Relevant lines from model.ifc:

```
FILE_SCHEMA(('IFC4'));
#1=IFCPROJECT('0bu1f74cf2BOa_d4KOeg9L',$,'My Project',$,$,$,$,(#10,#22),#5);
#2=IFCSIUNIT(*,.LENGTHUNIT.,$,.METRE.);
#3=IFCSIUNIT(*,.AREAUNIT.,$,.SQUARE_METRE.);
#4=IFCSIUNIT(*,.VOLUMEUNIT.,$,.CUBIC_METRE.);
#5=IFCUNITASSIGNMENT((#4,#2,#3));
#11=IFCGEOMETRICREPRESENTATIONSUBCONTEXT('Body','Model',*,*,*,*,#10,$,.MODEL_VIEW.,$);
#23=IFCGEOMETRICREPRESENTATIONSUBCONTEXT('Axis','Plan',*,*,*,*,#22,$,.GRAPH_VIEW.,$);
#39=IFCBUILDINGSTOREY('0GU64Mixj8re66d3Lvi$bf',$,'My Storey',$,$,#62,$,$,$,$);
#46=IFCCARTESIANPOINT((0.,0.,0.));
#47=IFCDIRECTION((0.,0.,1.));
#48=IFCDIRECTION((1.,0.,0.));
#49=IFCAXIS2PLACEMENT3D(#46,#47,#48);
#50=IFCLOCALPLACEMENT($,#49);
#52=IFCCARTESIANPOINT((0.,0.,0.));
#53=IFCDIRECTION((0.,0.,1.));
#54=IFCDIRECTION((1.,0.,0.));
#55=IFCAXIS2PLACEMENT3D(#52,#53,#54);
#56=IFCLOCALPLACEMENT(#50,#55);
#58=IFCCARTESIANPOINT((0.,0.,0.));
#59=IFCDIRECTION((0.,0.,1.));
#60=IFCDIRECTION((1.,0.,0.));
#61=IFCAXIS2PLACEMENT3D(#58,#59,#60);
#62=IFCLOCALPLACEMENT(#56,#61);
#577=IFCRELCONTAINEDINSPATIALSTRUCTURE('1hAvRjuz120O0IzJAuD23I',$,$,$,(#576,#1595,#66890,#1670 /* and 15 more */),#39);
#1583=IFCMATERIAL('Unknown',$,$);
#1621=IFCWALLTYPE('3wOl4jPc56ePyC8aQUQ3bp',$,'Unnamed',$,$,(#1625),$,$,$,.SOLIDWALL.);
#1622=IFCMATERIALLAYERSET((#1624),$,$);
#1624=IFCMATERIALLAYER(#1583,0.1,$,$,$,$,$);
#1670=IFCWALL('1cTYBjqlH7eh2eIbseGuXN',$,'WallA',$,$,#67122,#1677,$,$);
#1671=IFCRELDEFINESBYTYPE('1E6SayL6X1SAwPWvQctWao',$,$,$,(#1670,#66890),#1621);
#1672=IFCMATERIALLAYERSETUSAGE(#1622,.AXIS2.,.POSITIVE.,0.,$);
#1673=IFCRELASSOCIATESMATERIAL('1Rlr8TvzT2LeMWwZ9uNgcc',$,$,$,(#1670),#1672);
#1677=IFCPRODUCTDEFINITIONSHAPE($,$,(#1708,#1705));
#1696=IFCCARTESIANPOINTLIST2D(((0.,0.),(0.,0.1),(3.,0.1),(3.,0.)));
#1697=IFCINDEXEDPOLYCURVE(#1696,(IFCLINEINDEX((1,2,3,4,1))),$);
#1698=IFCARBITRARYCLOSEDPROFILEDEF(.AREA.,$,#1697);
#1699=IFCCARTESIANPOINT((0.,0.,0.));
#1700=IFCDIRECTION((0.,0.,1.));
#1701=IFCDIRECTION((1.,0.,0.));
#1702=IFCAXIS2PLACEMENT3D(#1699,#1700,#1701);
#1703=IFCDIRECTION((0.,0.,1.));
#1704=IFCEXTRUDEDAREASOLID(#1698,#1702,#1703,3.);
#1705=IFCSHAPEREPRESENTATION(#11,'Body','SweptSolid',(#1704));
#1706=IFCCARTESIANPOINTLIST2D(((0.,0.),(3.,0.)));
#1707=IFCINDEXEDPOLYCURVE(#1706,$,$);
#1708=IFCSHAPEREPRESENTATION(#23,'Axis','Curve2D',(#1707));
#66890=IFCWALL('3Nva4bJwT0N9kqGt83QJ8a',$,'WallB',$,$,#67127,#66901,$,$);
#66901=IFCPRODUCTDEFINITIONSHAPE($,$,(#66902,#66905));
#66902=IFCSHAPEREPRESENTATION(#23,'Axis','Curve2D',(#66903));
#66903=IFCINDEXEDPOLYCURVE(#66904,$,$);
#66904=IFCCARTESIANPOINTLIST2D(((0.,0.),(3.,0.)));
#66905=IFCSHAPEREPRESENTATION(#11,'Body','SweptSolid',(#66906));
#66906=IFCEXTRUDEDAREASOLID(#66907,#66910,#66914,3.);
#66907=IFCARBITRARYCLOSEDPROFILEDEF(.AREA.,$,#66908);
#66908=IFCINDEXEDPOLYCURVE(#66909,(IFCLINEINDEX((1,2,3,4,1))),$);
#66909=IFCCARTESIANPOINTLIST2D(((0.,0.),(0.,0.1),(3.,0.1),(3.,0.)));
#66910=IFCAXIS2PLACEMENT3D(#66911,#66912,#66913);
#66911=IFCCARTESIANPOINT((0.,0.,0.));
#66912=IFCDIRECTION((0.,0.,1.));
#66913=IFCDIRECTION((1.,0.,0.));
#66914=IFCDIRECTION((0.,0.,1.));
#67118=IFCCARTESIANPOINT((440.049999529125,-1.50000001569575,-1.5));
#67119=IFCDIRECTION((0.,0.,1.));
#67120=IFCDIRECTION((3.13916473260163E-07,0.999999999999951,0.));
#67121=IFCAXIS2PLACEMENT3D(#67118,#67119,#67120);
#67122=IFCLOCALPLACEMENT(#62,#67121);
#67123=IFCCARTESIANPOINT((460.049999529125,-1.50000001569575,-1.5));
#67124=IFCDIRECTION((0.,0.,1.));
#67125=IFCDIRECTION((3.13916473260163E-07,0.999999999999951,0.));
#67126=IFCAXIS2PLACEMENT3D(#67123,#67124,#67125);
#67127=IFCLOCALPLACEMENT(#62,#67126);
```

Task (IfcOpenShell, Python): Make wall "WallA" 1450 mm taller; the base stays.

```python
import ifcopenshell
import ifcopenshell.geom
import ifcopenshell.util.representation
import ifcopenshell.util.shape

model = ifcopenshell.open("model.ifc")
settings = ifcopenshell.geom.settings()


def volume(element):
    """Net volume in cubic metres, openings subtracted."""
    shape = ifcopenshell.geom.create_shape(settings, element)
    return ifcopenshell.util.shape.get_volume(shape.geometry)


wall = model.by_id(1670)
before = volume(wall)

body = ifcopenshell.util.representation.get_representation(wall, "Model", "Body")
solid = body.Items[0]
old_height = solid.Depth
solid.Depth += 1.45
after = volume(wall)

print(f"height {old_height:g} -> {solid.Depth:g}, volume {before:.3f} -> {after:.3f} m3")

model.write("model_v2.ifc")
```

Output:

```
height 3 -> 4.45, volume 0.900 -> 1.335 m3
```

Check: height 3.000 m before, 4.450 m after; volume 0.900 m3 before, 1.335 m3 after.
